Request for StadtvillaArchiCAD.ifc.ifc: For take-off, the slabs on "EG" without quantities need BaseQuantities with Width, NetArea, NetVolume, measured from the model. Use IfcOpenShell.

First a look at what the model holds.

```python
import ifcopenshell
import ifcopenshell.util.element
import ifcopenshell.util.unit

model = ifcopenshell.open("StadtvillaArchiCAD.ifc.ifc")
print(model.schema)
for unit_type in ("LENGTHUNIT", "AREAUNIT", "VOLUMEUNIT"):
    print(unit_type, ifcopenshell.util.unit.calculate_unit_scale(model, unit_type))
storey = next(s for s in model.by_type("IfcBuildingStorey") if s.Name == "EG")
slabs = [e for e in ifcopenshell.util.element.get_decomposition(storey) if e.is_a("IfcSlab")]
for e in sorted(slabs, key=lambda e: e.id()):
    print(e.id(), e.is_a(), e.Name, list(ifcopenshell.util.element.get_psets(e, qtos_only=True)), sep=" | ")
```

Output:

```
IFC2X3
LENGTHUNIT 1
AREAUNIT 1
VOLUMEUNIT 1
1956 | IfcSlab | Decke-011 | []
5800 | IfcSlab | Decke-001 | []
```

```python
import ifcopenshell
import ifcopenshell.api.pset
import ifcopenshell.geom
import ifcopenshell.util.element
import ifcopenshell.util.shape
import ifcopenshell.util.unit

model = ifcopenshell.open("StadtvillaArchiCAD.ifc.ifc")
unit_scale = ifcopenshell.util.unit.calculate_unit_scale(model)
area_scale = ifcopenshell.util.unit.calculate_unit_scale(model, "AREAUNIT")
volume_scale = ifcopenshell.util.unit.calculate_unit_scale(model, "VOLUMEUNIT")
settings = ifcopenshell.geom.settings()

storey = next(s for s in model.by_type("IfcBuildingStorey") if s.Name == "EG")
slabs = [e for e in ifcopenshell.util.element.get_decomposition(storey) if e.is_a("IfcSlab")]

for e in sorted(slabs, key=lambda e: e.id()):
    if ifcopenshell.util.element.get_psets(e, qtos_only=True, should_inherit=False):
        continue
    # Geometry comes back in metres, in the element's own axes.
    shape = ifcopenshell.geom.create_shape(settings, e)
    values = {
        "Width": ifcopenshell.util.shape.get_z(shape.geometry) / unit_scale,
        "NetArea": ifcopenshell.util.shape.get_footprint_area(shape.geometry) / area_scale,
        "NetVolume": ifcopenshell.util.shape.get_volume(shape.geometry) / volume_scale,
    }
    qto = ifcopenshell.api.pset.add_qto(model, product=e, name="BaseQuantities")
    ifcopenshell.api.pset.edit_qto(model, qto=qto, properties=values)
    print(e.id(), {k: round(v, 3) for k, v in values.items()})

model.write("StadtvillaArchiCAD.ifc_updated.ifc")
```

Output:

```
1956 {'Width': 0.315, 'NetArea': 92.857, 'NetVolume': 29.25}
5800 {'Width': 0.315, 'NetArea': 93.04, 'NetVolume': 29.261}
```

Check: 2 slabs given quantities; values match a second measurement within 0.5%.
